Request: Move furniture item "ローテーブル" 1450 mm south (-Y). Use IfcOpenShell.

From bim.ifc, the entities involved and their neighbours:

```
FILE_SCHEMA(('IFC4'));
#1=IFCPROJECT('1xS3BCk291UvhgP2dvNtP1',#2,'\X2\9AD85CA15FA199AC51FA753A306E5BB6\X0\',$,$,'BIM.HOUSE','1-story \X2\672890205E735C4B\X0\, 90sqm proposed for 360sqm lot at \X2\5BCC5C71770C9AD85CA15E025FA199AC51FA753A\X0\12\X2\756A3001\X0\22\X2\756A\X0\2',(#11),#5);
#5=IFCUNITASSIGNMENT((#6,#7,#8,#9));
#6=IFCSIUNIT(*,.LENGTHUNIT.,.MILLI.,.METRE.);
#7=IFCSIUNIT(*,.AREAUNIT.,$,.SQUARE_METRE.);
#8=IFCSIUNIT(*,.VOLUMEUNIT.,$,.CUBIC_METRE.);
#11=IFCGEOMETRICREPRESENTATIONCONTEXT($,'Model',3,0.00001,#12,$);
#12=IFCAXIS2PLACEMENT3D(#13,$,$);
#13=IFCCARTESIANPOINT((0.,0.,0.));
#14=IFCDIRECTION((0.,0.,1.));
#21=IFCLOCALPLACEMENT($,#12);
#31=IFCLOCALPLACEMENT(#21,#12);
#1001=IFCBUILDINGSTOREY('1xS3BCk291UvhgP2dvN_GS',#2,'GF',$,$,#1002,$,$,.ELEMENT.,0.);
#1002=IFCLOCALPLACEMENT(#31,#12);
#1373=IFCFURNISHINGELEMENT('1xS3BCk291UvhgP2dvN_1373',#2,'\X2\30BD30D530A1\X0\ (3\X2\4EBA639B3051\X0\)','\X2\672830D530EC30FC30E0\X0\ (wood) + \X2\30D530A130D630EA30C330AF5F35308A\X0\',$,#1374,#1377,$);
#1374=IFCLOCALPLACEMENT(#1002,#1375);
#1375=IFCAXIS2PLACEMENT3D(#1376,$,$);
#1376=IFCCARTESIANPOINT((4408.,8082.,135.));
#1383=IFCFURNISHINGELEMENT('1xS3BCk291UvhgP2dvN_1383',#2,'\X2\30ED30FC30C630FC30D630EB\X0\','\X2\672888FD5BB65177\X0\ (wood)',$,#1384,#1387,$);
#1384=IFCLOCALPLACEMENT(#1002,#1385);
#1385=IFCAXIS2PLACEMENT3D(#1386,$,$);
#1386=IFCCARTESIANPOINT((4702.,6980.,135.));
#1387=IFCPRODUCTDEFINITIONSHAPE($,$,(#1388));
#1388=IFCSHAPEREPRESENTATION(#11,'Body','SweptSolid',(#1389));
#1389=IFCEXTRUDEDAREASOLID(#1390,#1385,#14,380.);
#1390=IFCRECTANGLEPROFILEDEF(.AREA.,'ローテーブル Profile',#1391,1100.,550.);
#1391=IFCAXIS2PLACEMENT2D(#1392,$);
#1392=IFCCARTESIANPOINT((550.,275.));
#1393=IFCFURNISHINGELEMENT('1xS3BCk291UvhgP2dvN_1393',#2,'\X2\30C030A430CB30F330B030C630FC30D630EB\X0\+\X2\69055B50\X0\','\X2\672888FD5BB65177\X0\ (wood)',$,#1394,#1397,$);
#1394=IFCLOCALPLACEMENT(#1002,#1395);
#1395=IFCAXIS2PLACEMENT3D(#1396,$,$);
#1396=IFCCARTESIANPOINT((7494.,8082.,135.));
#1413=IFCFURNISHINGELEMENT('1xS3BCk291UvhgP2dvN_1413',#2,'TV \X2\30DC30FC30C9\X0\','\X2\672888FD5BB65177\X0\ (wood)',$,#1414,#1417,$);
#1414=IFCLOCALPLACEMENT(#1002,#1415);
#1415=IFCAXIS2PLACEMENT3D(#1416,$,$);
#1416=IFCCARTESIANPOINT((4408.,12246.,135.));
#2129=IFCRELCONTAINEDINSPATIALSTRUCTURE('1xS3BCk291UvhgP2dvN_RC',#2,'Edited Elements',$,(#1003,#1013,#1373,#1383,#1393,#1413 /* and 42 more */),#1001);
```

```python
import ifcopenshell
import ifcopenshell.api.geometry
import ifcopenshell.util.placement

model = ifcopenshell.open("bim.ifc")

item = model.by_guid("1xS3BCk291UvhgP2dvN_1383")
matrix = ifcopenshell.util.placement.get_local_placement(item.ObjectPlacement)
matrix[1, 3] -= 1450.0
ifcopenshell.api.geometry.edit_object_placement(model, product=item, matrix=matrix, is_si=False)

print(ifcopenshell.util.placement.get_local_placement(item.ObjectPlacement).round(3) + 0.0)

model.write("bim_updated.ifc")
```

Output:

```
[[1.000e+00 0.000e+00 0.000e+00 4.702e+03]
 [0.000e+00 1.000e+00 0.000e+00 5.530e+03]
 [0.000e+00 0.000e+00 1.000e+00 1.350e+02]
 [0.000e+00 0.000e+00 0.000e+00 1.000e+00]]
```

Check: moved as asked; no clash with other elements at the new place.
